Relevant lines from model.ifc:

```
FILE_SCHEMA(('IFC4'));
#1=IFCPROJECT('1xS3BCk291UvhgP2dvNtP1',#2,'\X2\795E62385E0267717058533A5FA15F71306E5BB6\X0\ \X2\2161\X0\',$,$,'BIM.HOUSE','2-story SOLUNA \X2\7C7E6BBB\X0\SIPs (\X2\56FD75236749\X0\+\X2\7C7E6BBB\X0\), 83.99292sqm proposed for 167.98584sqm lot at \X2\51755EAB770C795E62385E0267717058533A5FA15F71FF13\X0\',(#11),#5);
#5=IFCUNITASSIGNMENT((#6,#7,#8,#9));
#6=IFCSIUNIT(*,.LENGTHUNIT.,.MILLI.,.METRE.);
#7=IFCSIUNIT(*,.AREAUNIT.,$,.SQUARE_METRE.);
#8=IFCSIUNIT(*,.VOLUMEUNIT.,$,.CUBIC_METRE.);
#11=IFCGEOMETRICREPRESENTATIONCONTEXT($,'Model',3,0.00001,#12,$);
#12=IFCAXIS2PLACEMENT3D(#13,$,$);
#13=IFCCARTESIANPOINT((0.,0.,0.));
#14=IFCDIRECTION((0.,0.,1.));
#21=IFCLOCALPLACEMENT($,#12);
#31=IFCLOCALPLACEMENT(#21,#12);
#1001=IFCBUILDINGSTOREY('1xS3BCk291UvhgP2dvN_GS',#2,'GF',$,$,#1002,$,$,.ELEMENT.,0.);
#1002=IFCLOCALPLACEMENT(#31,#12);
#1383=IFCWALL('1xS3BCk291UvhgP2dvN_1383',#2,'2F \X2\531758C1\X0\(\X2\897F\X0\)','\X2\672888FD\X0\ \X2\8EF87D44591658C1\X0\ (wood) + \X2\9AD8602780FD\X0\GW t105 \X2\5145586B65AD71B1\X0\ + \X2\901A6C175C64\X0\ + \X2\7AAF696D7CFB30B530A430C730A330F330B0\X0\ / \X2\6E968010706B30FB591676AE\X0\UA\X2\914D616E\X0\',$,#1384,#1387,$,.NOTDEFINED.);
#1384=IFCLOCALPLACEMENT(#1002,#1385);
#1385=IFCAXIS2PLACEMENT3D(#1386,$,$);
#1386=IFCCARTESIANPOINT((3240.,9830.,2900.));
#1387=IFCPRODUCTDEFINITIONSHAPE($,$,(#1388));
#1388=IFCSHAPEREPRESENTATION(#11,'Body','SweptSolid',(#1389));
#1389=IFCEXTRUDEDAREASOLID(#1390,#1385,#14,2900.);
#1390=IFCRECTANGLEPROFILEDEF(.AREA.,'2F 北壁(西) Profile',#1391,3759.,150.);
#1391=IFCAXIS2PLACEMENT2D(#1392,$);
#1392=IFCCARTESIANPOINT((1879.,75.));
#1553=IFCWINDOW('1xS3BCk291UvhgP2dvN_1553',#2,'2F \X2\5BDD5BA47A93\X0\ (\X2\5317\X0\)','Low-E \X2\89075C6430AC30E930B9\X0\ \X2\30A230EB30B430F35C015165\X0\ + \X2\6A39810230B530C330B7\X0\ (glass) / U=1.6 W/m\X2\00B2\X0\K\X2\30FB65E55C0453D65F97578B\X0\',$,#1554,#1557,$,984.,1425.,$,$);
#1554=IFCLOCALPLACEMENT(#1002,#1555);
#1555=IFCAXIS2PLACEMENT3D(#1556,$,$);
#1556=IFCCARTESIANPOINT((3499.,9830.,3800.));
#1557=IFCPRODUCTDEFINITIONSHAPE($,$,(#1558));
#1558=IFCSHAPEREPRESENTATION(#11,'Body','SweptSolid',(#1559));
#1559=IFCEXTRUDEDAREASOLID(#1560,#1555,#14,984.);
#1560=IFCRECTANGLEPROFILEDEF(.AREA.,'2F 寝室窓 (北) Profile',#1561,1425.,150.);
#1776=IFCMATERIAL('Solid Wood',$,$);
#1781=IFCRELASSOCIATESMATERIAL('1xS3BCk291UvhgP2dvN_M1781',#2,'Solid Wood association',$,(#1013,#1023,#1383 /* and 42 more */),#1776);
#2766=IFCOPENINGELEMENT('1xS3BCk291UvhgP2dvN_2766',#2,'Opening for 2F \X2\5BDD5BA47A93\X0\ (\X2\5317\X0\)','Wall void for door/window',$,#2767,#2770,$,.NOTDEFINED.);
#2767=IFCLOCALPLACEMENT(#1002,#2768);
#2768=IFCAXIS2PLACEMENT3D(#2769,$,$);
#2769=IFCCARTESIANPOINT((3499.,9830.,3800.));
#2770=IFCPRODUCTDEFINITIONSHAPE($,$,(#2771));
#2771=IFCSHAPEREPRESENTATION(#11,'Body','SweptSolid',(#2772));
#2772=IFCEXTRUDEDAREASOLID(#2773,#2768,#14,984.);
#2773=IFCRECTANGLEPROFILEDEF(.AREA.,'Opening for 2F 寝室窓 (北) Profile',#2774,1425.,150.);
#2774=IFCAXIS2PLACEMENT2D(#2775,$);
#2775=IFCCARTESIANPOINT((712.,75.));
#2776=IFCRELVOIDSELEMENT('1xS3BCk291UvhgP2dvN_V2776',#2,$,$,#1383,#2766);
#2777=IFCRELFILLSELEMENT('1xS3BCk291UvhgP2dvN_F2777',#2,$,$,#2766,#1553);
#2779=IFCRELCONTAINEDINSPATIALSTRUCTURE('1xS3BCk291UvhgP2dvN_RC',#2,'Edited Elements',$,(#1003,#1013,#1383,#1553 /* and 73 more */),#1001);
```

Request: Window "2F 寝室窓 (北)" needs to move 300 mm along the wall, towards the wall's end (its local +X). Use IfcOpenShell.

```python
import ifcopenshell
import ifcopenshell.api.geometry
import ifcopenshell.util.placement

model = ifcopenshell.open("model.ifc")

window = model.by_guid("1xS3BCk291UvhgP2dvN_1553")
opening = window.FillsVoids[0].RelatingOpeningElement
wall = opening.VoidsElements[0].RelatingBuildingElement

wall_matrix = ifcopenshell.util.placement.get_local_placement(wall.ObjectPlacement)
shift = wall_matrix[:3, 0] * 300.0
before = ifcopenshell.util.placement.get_local_placement(window.ObjectPlacement)[:3, 3].copy()

# The window is not placed relative to its opening, so move both.
for product in (opening, window):
    matrix = ifcopenshell.util.placement.get_local_placement(product.ObjectPlacement)
    matrix[:3, 3] += shift
    ifcopenshell.api.geometry.edit_object_placement(model, product=product, matrix=matrix, is_si=False)

after = ifcopenshell.util.placement.get_local_placement(window.ObjectPlacement)[:3, 3]
print("window moved by", (after - before).round(3) + 0.0)

model.write("model_v2.ifc")
```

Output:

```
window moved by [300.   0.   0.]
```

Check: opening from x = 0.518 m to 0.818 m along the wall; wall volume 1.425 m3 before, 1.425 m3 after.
